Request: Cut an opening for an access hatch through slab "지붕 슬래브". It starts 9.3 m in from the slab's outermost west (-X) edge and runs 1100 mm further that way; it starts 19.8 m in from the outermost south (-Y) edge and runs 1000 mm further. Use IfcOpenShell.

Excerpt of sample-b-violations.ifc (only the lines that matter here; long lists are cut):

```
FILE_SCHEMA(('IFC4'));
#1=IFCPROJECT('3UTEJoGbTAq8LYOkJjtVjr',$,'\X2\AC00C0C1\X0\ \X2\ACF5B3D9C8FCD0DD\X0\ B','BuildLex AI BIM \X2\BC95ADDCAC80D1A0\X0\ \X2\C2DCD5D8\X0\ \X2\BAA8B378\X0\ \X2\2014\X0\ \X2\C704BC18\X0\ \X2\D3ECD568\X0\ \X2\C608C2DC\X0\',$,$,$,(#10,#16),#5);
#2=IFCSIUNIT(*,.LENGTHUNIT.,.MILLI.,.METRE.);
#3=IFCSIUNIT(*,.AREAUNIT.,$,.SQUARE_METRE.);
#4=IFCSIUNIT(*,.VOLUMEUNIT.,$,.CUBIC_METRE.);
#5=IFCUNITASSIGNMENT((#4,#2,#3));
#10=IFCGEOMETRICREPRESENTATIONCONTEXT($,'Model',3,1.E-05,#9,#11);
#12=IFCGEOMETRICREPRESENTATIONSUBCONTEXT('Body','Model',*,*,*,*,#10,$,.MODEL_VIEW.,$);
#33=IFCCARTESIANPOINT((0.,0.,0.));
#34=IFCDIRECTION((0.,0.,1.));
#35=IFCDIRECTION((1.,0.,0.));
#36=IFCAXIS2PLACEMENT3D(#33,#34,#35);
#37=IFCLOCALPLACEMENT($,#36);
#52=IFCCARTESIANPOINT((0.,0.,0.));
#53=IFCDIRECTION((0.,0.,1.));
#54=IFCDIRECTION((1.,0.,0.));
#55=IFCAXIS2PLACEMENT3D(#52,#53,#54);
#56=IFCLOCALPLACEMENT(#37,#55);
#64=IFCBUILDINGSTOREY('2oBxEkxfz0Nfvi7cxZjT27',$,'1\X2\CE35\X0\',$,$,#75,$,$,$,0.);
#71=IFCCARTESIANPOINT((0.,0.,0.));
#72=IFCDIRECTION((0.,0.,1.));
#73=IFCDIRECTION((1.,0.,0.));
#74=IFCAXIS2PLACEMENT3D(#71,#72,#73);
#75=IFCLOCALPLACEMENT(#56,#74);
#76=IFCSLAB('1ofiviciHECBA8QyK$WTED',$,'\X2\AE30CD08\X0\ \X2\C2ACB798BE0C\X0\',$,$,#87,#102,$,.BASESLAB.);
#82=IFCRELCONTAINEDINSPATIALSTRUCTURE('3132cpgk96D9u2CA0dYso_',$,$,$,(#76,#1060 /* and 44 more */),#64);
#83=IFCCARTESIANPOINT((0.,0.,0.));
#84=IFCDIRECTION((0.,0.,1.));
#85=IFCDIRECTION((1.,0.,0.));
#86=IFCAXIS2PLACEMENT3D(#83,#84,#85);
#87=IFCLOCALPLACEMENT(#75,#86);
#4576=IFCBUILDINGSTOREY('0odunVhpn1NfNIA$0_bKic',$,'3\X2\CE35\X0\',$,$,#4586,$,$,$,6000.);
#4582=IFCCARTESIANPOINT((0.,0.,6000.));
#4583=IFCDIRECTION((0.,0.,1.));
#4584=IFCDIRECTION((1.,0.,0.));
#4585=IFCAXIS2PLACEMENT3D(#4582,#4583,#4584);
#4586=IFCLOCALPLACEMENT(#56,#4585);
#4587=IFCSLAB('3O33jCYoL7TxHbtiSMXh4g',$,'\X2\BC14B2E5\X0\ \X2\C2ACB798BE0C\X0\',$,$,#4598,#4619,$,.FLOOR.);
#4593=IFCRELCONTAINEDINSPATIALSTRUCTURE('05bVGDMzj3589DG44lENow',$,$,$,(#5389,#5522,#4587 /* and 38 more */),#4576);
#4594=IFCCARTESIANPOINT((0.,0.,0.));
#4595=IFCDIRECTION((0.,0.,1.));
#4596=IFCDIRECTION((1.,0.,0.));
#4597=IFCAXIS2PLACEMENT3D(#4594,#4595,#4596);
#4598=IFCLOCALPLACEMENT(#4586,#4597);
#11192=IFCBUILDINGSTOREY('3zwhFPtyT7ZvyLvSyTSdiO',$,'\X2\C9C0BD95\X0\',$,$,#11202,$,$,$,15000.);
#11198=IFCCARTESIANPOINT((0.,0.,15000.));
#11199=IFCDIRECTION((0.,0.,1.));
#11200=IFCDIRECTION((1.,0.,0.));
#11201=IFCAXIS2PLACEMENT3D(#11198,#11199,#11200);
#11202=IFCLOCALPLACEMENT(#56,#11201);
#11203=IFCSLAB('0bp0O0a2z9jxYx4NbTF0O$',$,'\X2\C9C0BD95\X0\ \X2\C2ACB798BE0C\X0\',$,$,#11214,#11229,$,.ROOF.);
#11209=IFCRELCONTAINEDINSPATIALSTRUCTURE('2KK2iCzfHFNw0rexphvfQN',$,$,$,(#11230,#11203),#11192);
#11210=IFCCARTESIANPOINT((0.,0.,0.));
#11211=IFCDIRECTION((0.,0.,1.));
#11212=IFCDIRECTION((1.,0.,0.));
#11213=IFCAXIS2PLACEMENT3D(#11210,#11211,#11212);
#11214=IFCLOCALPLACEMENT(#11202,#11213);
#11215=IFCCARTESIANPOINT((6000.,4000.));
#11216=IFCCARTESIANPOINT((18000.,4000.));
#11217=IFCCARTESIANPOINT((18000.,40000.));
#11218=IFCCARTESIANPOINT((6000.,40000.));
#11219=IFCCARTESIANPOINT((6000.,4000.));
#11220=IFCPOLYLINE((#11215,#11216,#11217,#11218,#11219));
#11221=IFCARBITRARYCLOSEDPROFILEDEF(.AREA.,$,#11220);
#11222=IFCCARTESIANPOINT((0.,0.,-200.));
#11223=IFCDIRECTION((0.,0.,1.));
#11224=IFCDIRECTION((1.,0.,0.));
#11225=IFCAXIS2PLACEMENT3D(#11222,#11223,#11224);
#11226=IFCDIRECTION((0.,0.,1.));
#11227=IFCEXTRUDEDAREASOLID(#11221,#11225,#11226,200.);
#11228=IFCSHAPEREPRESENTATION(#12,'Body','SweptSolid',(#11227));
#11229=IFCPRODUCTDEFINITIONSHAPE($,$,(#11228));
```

```python
import numpy as np
import ifcopenshell
import ifcopenshell.api.feature
import ifcopenshell.api.geometry
import ifcopenshell.api.root
import ifcopenshell.geom
import ifcopenshell.util.placement
import ifcopenshell.util.representation
import ifcopenshell.util.shape
import ifcopenshell.util.unit

model = ifcopenshell.open("sample-b-violations.ifc")
unit_scale = ifcopenshell.util.unit.calculate_unit_scale(model)
settings = ifcopenshell.geom.settings()


def volume(element):
    """Net volume in cubic metres, openings subtracted."""
    shape = ifcopenshell.geom.create_shape(settings, element)
    return ifcopenshell.util.shape.get_volume(shape.geometry)


slab = model.by_guid("0bp0O0a2z9jxYx4NbTF0O$")
before = volume(slab)

# Extent in the slab's own axes, in metres. The edges named are its -X and -Y sides.
slab_shape = ifcopenshell.geom.create_shape(settings, slab)
vertices = ifcopenshell.util.shape.get_vertices(slab_shape.geometry)
x_min, y_min, bottom = vertices.min(axis=0)
top = vertices[:, 2].max()

opening = ifcopenshell.api.root.create_entity(model, ifc_class="IfcOpeningElement", name="Access hatch opening", predefined_type="OPENING")
context = ifcopenshell.util.representation.get_context(model, "Model", "Body", "MODEL_VIEW")
width, depth = 1.1, 1
outline = [(0.0, 0.0), (width, 0.0), (width, depth), (0.0, depth), (0.0, 0.0)]
# Overshoot both faces by 50 mm so the cut is clean.
shape = ifcopenshell.api.geometry.add_slab_representation(
    model, context=context, depth=top - bottom + 0.1, polyline=outline
)
ifcopenshell.api.geometry.assign_representation(model, product=opening, representation=shape)

matrix = ifcopenshell.util.placement.get_local_placement(slab.ObjectPlacement)
matrix[:, 3] = matrix @ np.append(np.array([x_min + 9.3, y_min + 19.8, bottom - 0.05]) / unit_scale, 1.0)
ifcopenshell.api.geometry.edit_object_placement(model, product=opening, matrix=matrix, is_si=False)
ifcopenshell.api.feature.add_feature(model, feature=opening, element=slab)

after = volume(slab)

print(f"slab volume {before:.3f} -> {after:.3f} m3")

model.write("sample-b-violations_v2.ifc")
```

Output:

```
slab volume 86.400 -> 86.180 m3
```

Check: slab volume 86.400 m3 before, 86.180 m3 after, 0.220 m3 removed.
